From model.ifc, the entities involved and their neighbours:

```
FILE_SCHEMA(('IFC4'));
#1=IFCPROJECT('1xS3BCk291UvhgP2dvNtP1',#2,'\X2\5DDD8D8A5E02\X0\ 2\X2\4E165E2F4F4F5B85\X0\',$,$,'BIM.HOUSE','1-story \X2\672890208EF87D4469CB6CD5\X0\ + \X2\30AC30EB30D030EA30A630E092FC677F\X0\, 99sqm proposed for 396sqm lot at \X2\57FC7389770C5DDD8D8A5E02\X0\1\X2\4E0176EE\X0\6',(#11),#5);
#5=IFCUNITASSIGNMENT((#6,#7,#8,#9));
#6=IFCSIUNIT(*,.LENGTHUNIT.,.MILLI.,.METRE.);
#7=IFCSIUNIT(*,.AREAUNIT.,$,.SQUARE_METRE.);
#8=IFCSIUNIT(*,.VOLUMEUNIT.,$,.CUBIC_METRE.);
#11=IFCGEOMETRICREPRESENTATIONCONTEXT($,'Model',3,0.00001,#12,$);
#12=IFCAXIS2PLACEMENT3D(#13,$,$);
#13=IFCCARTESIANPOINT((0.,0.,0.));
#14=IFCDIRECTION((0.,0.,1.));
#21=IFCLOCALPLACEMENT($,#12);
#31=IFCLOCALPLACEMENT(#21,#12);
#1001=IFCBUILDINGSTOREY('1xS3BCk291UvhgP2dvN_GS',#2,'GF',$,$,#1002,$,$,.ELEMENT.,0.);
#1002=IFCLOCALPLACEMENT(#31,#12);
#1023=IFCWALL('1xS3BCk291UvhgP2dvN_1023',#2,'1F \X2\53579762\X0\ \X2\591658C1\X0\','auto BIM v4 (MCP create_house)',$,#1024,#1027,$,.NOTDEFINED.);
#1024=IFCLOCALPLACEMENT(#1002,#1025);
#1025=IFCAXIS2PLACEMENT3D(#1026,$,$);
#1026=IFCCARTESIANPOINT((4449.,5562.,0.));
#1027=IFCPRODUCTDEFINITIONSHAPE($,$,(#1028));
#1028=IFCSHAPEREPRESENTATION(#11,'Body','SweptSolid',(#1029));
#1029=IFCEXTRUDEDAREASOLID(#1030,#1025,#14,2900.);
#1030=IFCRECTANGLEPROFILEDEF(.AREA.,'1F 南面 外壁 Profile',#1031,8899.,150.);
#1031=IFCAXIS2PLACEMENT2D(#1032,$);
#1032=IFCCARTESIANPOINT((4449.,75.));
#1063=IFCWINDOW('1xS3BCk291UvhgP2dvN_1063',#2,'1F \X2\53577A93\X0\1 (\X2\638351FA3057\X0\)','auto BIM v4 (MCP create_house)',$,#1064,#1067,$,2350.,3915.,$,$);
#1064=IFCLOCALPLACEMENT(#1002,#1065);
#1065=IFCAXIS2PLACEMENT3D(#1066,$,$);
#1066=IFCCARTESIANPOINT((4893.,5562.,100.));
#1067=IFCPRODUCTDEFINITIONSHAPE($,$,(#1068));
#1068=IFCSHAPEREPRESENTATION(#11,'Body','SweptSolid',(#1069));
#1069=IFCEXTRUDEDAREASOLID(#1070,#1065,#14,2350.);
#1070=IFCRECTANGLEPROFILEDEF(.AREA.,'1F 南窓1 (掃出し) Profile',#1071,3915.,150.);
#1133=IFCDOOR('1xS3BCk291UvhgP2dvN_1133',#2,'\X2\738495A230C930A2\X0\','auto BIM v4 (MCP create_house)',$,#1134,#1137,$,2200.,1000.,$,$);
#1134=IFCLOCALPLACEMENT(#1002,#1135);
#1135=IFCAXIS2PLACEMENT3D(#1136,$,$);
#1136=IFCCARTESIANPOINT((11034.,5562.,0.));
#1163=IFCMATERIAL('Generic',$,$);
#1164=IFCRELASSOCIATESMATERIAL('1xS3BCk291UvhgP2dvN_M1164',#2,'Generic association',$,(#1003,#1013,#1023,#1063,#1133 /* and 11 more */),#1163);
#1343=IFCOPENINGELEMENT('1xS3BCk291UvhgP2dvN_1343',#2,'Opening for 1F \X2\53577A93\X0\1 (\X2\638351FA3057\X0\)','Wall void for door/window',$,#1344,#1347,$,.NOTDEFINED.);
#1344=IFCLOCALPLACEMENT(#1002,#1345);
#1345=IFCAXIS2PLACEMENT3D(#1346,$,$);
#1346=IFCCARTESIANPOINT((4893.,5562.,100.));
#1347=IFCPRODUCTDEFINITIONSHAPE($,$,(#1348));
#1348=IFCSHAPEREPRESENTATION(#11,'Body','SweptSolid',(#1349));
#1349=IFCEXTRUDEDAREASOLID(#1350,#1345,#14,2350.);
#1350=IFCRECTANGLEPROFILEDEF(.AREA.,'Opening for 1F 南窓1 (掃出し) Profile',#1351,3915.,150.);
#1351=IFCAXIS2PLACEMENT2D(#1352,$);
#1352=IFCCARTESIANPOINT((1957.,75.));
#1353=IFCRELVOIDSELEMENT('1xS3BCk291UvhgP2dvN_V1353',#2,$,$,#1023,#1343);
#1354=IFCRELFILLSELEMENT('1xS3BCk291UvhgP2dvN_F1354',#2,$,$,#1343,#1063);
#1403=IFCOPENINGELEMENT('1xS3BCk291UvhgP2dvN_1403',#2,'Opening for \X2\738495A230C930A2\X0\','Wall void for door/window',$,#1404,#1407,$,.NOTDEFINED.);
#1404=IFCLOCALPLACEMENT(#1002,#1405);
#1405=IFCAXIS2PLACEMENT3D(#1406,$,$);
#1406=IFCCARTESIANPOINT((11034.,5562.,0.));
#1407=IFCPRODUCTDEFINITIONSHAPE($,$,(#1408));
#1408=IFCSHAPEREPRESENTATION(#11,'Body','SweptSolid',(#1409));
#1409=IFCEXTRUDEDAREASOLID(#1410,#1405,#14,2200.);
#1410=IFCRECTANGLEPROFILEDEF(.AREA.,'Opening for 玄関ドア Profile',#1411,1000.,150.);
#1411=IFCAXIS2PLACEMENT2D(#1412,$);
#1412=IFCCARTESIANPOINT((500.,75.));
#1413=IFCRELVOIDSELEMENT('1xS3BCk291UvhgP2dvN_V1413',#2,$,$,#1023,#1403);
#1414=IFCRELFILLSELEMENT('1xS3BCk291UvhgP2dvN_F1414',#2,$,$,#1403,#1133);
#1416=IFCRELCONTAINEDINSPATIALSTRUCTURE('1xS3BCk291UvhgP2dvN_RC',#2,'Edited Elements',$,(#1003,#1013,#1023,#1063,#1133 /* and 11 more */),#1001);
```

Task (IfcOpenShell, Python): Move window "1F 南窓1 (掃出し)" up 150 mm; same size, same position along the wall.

```python
import numpy as np
import ifcopenshell
import ifcopenshell.api.geometry
import ifcopenshell.util.placement
import ifcopenshell.util.unit

model = ifcopenshell.open("model.ifc")
unit_scale = ifcopenshell.util.unit.calculate_unit_scale(model)

window = model.by_guid("1xS3BCk291UvhgP2dvN_1063")
opening = window.FillsVoids[0].RelatingOpeningElement
dz = 0.15 / unit_scale

shift = np.array([0.0, 0.0, dz])
# The window is not placed relative to its opening, so move both.
for product in (opening, window):
    matrix = ifcopenshell.util.placement.get_local_placement(product.ObjectPlacement)
    matrix[:3, 3] += shift
    ifcopenshell.api.geometry.edit_object_placement(model, product=product, matrix=matrix, is_si=False)

print(f"moved by {dz * unit_scale:+.3f} m")

model.write("model-out.ifc")
```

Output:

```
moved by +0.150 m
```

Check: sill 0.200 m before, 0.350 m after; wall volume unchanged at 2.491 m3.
